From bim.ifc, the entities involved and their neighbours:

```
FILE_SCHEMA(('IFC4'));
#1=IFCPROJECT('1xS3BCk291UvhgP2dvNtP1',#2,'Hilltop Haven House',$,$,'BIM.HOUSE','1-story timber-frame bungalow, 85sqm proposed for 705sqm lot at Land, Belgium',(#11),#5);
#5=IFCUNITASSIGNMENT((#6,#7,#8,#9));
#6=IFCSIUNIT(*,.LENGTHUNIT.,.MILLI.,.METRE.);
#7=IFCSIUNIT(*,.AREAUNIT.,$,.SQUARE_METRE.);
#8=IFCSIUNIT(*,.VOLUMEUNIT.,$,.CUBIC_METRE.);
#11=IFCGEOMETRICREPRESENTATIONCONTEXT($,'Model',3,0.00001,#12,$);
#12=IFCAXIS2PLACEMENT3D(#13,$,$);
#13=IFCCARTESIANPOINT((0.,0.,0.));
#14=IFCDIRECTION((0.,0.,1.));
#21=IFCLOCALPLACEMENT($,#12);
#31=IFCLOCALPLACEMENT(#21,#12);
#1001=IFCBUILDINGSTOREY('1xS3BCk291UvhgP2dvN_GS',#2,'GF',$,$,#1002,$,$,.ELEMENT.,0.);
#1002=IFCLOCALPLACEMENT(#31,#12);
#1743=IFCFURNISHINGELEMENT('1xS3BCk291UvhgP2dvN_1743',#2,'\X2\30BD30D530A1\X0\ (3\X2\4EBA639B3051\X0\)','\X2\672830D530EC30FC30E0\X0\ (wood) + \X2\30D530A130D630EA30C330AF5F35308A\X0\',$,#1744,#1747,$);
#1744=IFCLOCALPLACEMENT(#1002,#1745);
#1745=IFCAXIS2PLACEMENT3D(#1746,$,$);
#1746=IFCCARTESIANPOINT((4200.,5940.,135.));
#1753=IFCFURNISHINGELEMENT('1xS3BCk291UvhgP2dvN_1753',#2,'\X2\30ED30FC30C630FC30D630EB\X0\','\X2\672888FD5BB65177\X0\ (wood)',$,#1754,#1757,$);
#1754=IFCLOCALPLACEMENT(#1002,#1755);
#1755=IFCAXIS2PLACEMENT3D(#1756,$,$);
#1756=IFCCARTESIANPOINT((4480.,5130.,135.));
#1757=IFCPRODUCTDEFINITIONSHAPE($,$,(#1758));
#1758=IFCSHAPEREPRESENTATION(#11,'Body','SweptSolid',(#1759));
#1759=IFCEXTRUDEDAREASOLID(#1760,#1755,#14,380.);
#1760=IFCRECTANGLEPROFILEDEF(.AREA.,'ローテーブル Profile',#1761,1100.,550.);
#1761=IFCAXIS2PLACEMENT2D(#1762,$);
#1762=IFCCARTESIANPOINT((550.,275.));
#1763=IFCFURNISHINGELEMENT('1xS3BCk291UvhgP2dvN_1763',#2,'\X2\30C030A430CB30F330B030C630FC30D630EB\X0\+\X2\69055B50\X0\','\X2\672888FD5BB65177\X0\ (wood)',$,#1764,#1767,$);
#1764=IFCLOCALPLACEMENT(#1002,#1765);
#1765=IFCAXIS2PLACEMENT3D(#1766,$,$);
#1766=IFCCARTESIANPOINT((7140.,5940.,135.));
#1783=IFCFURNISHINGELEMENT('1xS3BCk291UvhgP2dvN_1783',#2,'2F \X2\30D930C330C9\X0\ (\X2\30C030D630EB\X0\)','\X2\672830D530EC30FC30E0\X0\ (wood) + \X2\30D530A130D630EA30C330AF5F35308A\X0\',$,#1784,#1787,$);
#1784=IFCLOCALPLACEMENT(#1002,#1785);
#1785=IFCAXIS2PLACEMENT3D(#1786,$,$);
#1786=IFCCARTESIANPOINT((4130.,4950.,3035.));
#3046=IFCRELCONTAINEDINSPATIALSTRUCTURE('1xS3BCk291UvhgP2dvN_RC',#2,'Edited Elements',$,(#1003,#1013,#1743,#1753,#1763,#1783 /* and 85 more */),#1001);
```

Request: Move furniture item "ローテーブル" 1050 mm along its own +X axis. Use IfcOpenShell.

```python
import ifcopenshell
import ifcopenshell.api.geometry
import ifcopenshell.util.placement

model = ifcopenshell.open("bim.ifc")

item = model.by_guid("1xS3BCk291UvhgP2dvN_1753")
matrix = ifcopenshell.util.placement.get_local_placement(item.ObjectPlacement)
matrix[:3, 3] += matrix[:3, 0] * 1050.0
ifcopenshell.api.geometry.edit_object_placement(model, product=item, matrix=matrix, is_si=False)

print(ifcopenshell.util.placement.get_local_placement(item.ObjectPlacement).round(3) + 0.0)

model.write("bim_updated.ifc")
```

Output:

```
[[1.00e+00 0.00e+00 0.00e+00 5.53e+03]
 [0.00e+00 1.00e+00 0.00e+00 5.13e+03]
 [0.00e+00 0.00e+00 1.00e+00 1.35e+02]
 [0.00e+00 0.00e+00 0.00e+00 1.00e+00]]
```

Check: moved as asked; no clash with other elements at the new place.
